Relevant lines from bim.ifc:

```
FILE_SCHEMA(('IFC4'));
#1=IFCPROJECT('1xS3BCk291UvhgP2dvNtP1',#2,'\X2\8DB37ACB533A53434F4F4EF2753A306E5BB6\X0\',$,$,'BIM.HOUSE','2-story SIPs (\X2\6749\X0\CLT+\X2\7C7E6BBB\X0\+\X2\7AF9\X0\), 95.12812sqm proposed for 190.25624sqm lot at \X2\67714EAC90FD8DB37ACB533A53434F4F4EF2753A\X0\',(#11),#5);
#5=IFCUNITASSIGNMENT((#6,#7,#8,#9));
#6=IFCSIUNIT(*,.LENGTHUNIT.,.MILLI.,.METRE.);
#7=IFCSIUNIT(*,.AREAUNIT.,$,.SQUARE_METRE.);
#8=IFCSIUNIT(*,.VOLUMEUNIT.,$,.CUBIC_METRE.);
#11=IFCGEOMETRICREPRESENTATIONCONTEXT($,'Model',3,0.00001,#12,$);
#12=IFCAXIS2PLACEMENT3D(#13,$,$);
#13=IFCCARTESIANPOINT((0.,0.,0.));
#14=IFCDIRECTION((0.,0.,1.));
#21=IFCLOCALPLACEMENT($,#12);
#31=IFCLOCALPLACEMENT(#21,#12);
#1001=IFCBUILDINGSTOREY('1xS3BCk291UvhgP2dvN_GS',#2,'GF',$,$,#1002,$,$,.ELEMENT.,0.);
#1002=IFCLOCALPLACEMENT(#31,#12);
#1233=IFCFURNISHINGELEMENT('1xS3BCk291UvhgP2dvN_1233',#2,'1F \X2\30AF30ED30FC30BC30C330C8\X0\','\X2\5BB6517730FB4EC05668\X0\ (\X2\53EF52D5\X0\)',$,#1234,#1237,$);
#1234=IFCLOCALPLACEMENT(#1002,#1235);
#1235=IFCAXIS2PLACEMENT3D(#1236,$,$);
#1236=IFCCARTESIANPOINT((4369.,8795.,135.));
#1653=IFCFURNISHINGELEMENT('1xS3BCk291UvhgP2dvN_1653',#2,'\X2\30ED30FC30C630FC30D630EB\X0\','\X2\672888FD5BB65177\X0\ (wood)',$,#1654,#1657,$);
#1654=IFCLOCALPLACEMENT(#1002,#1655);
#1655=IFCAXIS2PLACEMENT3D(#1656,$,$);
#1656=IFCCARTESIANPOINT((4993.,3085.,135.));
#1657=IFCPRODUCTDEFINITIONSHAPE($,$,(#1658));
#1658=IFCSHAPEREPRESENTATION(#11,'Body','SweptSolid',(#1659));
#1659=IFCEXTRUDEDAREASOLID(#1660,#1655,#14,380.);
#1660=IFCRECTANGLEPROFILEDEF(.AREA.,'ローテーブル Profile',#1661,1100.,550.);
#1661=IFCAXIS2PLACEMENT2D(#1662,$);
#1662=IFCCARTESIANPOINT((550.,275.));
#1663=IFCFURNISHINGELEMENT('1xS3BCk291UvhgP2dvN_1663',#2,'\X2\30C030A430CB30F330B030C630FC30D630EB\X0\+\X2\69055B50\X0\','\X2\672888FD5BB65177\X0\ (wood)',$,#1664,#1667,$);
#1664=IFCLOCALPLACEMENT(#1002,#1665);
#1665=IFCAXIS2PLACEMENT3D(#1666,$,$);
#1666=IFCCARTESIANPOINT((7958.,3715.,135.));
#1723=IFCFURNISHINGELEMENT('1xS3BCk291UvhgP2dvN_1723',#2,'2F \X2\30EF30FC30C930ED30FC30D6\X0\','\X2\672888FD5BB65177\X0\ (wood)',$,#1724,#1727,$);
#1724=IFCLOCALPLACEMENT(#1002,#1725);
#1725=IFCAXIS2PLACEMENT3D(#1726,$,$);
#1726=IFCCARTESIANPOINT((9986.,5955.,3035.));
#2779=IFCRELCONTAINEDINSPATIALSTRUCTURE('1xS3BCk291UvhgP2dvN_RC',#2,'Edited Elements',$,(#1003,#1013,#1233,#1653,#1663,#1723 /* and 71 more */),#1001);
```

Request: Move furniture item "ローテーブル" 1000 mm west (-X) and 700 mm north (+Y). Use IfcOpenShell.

```python
import ifcopenshell
import ifcopenshell.api.geometry
import ifcopenshell.util.placement
import ifcopenshell.util.unit

model = ifcopenshell.open("bim.ifc")
unit_scale = ifcopenshell.util.unit.calculate_unit_scale(model)

item = model.by_id(1653)
matrix = ifcopenshell.util.placement.get_local_placement(item.ObjectPlacement)
matrix[0, 3] -= 1 / unit_scale
matrix[1, 3] += 0.7 / unit_scale
ifcopenshell.api.geometry.edit_object_placement(model, product=item, matrix=matrix, is_si=False)

print(ifcopenshell.util.placement.get_local_placement(item.ObjectPlacement).round(3) + 0.0)

model.write("bim_updated.ifc")
```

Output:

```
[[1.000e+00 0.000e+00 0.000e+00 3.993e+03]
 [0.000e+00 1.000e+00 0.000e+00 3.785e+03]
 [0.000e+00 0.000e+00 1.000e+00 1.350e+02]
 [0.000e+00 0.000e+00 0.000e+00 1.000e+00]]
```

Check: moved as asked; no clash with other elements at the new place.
